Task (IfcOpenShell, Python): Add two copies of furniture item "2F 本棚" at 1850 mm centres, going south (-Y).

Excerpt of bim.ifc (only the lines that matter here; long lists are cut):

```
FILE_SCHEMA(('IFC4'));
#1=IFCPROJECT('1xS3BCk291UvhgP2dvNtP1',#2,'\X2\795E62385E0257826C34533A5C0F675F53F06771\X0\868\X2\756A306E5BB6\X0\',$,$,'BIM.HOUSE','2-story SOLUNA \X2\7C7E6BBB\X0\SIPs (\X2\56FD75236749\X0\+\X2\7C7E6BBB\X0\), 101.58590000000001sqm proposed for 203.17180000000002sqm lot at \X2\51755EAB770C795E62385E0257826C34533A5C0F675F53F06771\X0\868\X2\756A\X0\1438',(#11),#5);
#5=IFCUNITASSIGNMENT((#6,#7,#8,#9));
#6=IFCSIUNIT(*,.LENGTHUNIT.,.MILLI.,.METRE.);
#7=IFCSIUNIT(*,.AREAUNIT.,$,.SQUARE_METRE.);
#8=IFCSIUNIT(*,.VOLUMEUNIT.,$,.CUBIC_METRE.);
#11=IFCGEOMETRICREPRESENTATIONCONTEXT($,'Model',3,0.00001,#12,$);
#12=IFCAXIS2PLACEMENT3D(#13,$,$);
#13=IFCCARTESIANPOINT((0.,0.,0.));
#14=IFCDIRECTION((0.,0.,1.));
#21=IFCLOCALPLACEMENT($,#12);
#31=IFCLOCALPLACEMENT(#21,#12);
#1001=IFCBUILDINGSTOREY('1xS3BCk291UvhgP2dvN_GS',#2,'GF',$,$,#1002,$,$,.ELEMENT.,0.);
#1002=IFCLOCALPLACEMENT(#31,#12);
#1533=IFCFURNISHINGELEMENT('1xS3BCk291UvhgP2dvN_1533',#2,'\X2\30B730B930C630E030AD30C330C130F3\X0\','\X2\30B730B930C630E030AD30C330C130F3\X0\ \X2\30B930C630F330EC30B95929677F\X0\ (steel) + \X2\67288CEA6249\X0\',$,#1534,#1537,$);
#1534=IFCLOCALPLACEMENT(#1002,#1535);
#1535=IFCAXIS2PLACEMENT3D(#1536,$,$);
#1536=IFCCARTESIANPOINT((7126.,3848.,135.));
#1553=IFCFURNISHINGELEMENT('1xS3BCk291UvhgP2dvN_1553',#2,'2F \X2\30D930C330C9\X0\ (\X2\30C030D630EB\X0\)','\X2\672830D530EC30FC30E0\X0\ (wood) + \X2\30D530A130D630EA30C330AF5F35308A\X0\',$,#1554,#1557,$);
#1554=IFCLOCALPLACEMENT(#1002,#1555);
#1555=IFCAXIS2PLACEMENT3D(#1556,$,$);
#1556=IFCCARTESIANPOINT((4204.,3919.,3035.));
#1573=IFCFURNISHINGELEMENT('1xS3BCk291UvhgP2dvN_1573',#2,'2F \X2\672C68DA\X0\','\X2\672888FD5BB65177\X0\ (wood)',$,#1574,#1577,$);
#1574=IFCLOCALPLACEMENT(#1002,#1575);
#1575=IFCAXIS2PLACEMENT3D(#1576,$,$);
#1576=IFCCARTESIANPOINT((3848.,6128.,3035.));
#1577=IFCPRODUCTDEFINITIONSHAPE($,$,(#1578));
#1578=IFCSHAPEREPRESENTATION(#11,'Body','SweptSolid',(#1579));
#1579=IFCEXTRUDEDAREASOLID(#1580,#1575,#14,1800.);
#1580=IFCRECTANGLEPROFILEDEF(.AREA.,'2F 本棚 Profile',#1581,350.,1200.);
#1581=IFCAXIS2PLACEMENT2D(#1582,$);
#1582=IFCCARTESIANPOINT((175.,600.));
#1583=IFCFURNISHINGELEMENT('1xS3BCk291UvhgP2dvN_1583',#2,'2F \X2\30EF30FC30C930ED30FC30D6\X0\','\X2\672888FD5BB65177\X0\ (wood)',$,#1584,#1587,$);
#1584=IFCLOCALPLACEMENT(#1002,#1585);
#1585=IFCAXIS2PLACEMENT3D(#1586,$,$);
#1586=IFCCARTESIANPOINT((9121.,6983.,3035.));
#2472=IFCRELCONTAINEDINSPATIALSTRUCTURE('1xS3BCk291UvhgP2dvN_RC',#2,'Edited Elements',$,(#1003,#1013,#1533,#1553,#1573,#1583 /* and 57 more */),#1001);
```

```python
import numpy as np
import ifcopenshell
import ifcopenshell.api.geometry
import ifcopenshell.api.root
import ifcopenshell.util.element
import ifcopenshell.util.placement
import ifcopenshell.util.unit

model = ifcopenshell.open("bim.ifc")
unit_scale = ifcopenshell.util.unit.calculate_unit_scale(model)


def reuse_history(source, copy):
    """copy_class also copies each property set's owner history, people and application; keep the originals."""
    for rel in copy.IsDefinedBy:
        if rel.is_a("IfcRelDefinesByProperties") and (history := rel.RelatingPropertyDefinition.OwnerHistory):
            rel.RelatingPropertyDefinition.OwnerHistory = source.OwnerHistory
            ifcopenshell.util.element.remove_deep2(model, history)


source = model.by_guid("1xS3BCk291UvhgP2dvN_1573")
base = ifcopenshell.util.placement.get_local_placement(source.ObjectPlacement)
step = np.array([0.0, -1.0, 0.0]) * 1.85 / unit_scale

for i in range(1, 3):
    copy = ifcopenshell.api.root.copy_class(model, product=source)
    copy.Representation = ifcopenshell.util.element.copy_deep(
        model, source.Representation, exclude=["IfcGeometricRepresentationContext", "IfcRepresentationMap"]
    )
    reuse_history(source, copy)
    matrix = base.copy()
    matrix[:3, 3] += i * step
    print("added at", matrix[:3, 3].round(3) + 0.0)
    ifcopenshell.api.geometry.edit_object_placement(model, product=copy, matrix=matrix, is_si=False)

model.write("bim-out.ifc")
```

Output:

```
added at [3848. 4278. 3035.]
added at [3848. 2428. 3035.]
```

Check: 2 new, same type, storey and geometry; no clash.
